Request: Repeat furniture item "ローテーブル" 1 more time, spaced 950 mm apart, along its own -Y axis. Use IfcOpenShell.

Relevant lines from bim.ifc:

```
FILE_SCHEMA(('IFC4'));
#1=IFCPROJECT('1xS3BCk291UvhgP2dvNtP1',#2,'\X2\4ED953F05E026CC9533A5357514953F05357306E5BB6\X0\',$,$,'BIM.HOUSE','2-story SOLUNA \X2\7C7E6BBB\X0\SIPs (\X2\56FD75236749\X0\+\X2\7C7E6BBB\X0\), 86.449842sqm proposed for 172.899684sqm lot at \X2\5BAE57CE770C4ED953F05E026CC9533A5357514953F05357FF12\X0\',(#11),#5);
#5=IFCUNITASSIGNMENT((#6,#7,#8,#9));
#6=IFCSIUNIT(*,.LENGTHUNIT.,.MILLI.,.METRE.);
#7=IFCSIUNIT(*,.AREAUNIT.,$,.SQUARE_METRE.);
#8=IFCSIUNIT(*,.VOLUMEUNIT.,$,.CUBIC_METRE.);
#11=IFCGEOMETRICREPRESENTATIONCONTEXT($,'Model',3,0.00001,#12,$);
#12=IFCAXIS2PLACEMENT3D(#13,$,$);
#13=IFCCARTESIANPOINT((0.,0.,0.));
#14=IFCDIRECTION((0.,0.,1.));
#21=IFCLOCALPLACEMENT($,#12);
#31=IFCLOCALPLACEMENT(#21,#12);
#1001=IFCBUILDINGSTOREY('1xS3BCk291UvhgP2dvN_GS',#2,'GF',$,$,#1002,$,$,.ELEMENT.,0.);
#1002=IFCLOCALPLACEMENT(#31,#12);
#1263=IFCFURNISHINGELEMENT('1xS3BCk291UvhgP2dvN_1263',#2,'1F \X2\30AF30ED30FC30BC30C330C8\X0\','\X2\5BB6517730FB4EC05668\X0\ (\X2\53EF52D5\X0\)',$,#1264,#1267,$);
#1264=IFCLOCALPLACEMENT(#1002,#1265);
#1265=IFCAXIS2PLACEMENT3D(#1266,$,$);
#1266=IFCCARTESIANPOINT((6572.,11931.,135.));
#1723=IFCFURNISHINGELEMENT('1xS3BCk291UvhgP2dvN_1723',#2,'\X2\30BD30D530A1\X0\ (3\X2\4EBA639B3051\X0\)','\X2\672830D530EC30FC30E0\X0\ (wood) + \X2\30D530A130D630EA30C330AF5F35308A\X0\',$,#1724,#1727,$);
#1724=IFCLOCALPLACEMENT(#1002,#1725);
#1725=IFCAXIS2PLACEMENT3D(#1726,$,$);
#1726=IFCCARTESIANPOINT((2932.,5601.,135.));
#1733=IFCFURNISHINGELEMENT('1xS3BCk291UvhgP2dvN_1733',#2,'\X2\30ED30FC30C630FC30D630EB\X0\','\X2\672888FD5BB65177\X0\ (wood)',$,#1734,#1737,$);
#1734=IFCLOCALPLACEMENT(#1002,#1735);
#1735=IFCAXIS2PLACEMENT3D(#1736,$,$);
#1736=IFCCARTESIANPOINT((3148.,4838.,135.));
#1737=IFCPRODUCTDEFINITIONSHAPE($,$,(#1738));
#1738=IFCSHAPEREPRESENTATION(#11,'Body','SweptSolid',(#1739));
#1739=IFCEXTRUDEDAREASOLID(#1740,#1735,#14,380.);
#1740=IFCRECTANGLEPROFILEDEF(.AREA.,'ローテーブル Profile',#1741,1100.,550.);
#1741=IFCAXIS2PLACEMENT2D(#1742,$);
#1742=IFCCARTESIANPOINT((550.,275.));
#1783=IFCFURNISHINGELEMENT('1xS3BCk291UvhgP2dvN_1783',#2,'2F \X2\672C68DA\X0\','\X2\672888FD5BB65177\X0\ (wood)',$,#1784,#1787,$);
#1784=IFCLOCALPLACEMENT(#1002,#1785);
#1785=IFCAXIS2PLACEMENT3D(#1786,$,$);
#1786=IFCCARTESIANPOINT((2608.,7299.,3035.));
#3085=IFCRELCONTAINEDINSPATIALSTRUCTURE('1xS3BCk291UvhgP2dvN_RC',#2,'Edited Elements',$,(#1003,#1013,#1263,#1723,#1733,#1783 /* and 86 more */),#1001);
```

```python
import ifcopenshell
import ifcopenshell.api.geometry
import ifcopenshell.api.root
import ifcopenshell.util.element
import ifcopenshell.util.placement
import ifcopenshell.util.unit

model = ifcopenshell.open("bim.ifc")
unit_scale = ifcopenshell.util.unit.calculate_unit_scale(model)


def reuse_history(source, copy):
    """copy_class also copies each property set's owner history, people and application; keep the originals."""
    for rel in copy.IsDefinedBy:
        if rel.is_a("IfcRelDefinesByProperties") and (history := rel.RelatingPropertyDefinition.OwnerHistory):
            rel.RelatingPropertyDefinition.OwnerHistory = source.OwnerHistory
            ifcopenshell.util.element.remove_deep2(model, history)


source = model.by_guid("1xS3BCk291UvhgP2dvN_1733")
base = ifcopenshell.util.placement.get_local_placement(source.ObjectPlacement)
step = -base[:3, 1] * 0.95 / unit_scale

for i in range(1, 2):
    copy = ifcopenshell.api.root.copy_class(model, product=source)
    copy.Representation = ifcopenshell.util.element.copy_deep(
        model, source.Representation, exclude=["IfcGeometricRepresentationContext", "IfcRepresentationMap"]
    )
    reuse_history(source, copy)
    matrix = base.copy()
    matrix[:3, 3] += i * step
    print("added at", matrix[:3, 3].round(3) + 0.0)
    ifcopenshell.api.geometry.edit_object_placement(model, product=copy, matrix=matrix, is_si=False)

model.write("bim_v2.ifc")
```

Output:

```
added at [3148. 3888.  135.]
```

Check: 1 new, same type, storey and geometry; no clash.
